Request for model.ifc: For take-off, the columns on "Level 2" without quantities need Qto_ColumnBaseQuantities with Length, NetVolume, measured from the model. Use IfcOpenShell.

First a look at what the model holds.

```python
import ifcopenshell
import ifcopenshell.util.element
import ifcopenshell.util.unit

model = ifcopenshell.open("model.ifc")
print(model.schema)
for unit_type in ("LENGTHUNIT", "AREAUNIT", "VOLUMEUNIT"):
    print(unit_type, ifcopenshell.util.unit.calculate_unit_scale(model, unit_type))
storey = next(s for s in model.by_type("IfcBuildingStorey") if s.Name == "Level 2")
columns = [e for e in ifcopenshell.util.element.get_decomposition(storey) if e.is_a("IfcColumn")]
for e in sorted(columns, key=lambda e: e.id()):
    print(e.id(), e.is_a(), e.Name, list(ifcopenshell.util.element.get_psets(e, qtos_only=True)), sep=" | ")
```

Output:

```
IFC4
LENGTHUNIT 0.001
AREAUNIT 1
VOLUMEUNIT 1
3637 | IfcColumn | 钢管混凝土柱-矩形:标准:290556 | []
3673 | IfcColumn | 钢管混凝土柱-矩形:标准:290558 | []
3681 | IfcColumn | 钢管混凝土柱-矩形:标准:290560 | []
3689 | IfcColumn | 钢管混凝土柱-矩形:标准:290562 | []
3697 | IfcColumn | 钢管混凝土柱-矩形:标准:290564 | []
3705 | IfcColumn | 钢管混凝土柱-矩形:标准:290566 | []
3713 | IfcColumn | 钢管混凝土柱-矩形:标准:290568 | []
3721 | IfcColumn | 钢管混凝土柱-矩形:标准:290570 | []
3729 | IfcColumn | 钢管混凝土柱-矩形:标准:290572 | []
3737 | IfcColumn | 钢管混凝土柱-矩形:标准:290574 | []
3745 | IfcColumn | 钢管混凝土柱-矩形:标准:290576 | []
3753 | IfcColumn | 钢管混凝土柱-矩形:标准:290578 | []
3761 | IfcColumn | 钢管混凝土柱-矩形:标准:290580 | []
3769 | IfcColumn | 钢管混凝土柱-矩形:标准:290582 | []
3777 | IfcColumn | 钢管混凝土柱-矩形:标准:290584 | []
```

```python
import ifcopenshell
import ifcopenshell.api.pset
import ifcopenshell.geom
import ifcopenshell.util.element
import ifcopenshell.util.shape
import ifcopenshell.util.unit

model = ifcopenshell.open("model.ifc")
unit_scale = ifcopenshell.util.unit.calculate_unit_scale(model)
volume_scale = ifcopenshell.util.unit.calculate_unit_scale(model, "VOLUMEUNIT")
settings = ifcopenshell.geom.settings()

storey = next(s for s in model.by_type("IfcBuildingStorey") if s.Name == "Level 2")
columns = [e for e in ifcopenshell.util.element.get_decomposition(storey) if e.is_a("IfcColumn")]

for e in sorted(columns, key=lambda e: e.id()):
    if ifcopenshell.util.element.get_psets(e, qtos_only=True, should_inherit=False):
        continue
    # Geometry comes back in metres, in the element's own axes.
    shape = ifcopenshell.geom.create_shape(settings, e)
    values = {
        "Length": ifcopenshell.util.shape.get_z(shape.geometry) / unit_scale,
        "NetVolume": ifcopenshell.util.shape.get_volume(shape.geometry) / volume_scale,
    }
    qto = ifcopenshell.api.pset.add_qto(model, product=e, name="Qto_ColumnBaseQuantities")
    ifcopenshell.api.pset.edit_qto(model, qto=qto, properties=values)
    print(e.id(), {k: round(v, 3) for k, v in values.items()})

model.write("model_rev.ifc")
```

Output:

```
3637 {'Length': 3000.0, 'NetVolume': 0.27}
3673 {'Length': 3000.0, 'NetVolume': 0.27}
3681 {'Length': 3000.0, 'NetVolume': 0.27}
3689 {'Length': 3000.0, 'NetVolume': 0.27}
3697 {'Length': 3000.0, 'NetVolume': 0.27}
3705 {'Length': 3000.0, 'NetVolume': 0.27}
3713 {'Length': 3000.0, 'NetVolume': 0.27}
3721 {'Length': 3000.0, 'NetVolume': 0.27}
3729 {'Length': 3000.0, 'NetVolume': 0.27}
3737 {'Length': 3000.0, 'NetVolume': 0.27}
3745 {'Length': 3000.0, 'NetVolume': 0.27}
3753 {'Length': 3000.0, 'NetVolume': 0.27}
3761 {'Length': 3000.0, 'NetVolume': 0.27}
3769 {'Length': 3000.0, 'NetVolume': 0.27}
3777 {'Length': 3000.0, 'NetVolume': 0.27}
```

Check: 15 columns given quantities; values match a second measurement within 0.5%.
